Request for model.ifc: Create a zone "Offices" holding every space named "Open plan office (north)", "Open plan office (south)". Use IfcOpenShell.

First a look at what the model holds.

```python
import ifcopenshell

model = ifcopenshell.open("model.ifc")
print(model.schema)
seen = {}
for space in model.by_type("IfcSpace"):
    seen[space.LongName] = seen.get(space.LongName, 0) + 1
for name, count in sorted(seen.items(), key=str):
    print(count, "x", name)
print("zones:", [z.Name for z in model.by_type("IfcZone")][:20])
```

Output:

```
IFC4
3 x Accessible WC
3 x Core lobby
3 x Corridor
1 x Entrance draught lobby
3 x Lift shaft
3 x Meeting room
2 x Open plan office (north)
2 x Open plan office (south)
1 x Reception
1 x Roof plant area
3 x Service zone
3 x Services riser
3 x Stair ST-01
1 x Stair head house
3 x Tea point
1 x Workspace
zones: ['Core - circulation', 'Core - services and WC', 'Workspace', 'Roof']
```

```python
import ifcopenshell
import ifcopenshell.api.group
import ifcopenshell.api.root

model = ifcopenshell.open("model.ifc")

names = {"Open plan office (north)", "Open plan office (south)"}
spaces = [s for s in model.by_type("IfcSpace") if s.LongName in names]

zone = ifcopenshell.api.root.create_entity(model, ifc_class="IfcZone", name="Offices")
ifcopenshell.api.group.assign_group(model, products=spaces, group=zone)
print(len(spaces), "spaces in", zone.Name)

model.write("model_updated.ifc")
```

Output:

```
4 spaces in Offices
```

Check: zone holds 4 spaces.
